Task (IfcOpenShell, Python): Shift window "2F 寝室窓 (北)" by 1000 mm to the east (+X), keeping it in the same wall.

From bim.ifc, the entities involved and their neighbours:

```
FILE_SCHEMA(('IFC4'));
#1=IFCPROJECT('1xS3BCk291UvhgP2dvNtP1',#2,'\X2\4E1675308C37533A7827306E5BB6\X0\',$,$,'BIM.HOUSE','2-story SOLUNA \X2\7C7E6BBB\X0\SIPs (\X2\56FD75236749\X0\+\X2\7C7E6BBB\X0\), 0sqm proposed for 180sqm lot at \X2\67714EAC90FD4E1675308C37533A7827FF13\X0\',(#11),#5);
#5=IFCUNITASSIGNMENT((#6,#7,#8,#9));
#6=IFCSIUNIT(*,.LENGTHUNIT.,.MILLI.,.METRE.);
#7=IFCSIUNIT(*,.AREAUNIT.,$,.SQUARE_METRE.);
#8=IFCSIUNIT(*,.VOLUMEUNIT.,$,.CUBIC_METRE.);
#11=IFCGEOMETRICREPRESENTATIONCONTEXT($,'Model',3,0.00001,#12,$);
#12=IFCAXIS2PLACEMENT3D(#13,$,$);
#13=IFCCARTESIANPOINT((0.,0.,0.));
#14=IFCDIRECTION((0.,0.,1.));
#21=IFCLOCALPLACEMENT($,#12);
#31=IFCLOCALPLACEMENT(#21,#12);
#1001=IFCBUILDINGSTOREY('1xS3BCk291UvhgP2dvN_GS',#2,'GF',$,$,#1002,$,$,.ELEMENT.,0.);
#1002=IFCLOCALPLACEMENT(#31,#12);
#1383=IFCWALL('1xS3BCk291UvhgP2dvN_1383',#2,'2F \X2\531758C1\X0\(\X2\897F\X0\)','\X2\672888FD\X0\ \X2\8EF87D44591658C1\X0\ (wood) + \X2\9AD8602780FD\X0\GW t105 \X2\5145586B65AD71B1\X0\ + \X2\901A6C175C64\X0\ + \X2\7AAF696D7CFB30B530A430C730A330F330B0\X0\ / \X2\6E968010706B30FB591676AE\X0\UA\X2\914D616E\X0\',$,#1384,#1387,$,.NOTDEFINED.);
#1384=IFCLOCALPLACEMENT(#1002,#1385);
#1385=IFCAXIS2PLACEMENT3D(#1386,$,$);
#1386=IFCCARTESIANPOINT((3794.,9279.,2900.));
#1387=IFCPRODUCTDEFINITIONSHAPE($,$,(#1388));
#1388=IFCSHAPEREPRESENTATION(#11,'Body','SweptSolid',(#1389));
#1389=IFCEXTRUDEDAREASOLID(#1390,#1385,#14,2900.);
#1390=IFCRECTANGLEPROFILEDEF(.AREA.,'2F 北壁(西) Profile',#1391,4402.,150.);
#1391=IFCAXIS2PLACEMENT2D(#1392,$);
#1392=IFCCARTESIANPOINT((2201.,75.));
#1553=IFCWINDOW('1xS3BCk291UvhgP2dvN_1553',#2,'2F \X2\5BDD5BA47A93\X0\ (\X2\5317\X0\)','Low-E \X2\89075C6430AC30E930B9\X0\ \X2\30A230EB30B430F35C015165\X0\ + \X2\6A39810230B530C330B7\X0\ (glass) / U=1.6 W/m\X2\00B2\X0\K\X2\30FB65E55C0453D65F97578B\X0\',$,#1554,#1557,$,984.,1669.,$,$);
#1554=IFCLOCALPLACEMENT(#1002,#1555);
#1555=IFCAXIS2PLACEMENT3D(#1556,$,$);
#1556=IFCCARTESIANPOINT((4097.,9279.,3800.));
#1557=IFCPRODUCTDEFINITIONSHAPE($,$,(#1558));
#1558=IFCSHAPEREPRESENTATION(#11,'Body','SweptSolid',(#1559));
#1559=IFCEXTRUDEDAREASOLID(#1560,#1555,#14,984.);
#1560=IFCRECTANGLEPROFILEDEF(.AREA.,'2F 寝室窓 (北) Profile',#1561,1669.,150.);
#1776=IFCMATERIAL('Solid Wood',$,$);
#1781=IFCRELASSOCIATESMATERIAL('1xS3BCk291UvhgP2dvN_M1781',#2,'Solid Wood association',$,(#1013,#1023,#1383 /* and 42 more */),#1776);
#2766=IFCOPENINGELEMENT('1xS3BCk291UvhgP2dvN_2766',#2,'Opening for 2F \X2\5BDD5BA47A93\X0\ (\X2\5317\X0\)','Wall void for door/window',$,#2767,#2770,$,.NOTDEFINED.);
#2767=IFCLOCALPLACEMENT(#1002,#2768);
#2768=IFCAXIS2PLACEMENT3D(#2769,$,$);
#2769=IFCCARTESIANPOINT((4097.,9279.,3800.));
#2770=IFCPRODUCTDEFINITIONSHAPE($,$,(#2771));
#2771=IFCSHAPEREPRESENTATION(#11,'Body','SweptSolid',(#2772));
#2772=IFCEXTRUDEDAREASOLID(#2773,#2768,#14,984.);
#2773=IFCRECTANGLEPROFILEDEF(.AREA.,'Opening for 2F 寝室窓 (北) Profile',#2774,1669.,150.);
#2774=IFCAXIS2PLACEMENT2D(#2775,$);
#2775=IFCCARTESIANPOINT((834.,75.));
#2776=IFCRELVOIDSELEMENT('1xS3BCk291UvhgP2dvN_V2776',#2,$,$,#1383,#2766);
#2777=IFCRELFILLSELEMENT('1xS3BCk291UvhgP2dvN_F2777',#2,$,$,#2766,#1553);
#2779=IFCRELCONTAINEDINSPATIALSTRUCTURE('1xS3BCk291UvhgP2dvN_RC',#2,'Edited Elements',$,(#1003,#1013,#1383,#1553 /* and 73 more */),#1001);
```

```python
import ifcopenshell
import ifcopenshell.api.geometry
import ifcopenshell.util.placement
import ifcopenshell.util.unit

model = ifcopenshell.open("bim.ifc")
unit_scale = ifcopenshell.util.unit.calculate_unit_scale(model)

window = model.by_guid("1xS3BCk291UvhgP2dvN_1553")
opening = window.FillsVoids[0].RelatingOpeningElement
wall = opening.VoidsElements[0].RelatingBuildingElement

wall_matrix = ifcopenshell.util.placement.get_local_placement(wall.ObjectPlacement)
shift = wall_matrix[:3, 0] * 1 / unit_scale
before = ifcopenshell.util.placement.get_local_placement(window.ObjectPlacement)[:3, 3].copy()

# The window is not placed relative to its opening, so move both.
for product in (opening, window):
    matrix = ifcopenshell.util.placement.get_local_placement(product.ObjectPlacement)
    matrix[:3, 3] += shift
    ifcopenshell.api.geometry.edit_object_placement(model, product=product, matrix=matrix, is_si=False)

after = ifcopenshell.util.placement.get_local_placement(window.ObjectPlacement)[:3, 3]
print("window moved by", (after - before).round(3) + 0.0)

model.write("bim_updated.ifc")
```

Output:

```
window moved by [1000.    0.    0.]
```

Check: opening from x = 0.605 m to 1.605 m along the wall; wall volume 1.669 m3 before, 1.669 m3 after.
